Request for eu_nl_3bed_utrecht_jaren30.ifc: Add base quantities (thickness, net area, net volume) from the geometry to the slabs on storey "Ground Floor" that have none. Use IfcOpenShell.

First a look at what the model holds.

```python
import ifcopenshell
import ifcopenshell.util.element
import ifcopenshell.util.unit

model = ifcopenshell.open("eu_nl_3bed_utrecht_jaren30.ifc")
print(model.schema)
for unit_type in ("LENGTHUNIT", "AREAUNIT", "VOLUMEUNIT"):
    print(unit_type, ifcopenshell.util.unit.calculate_unit_scale(model, unit_type))
storey = next(s for s in model.by_type("IfcBuildingStorey") if s.Name == "Ground Floor")
slabs = [e for e in ifcopenshell.util.element.get_decomposition(storey) if e.is_a("IfcSlab")]
for e in sorted(slabs, key=lambda e: e.id()):
    print(e.id(), e.is_a(), e.Name, list(ifcopenshell.util.element.get_psets(e, qtos_only=True)), sep=" | ")
```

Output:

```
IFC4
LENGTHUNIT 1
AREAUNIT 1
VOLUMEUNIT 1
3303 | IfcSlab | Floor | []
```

```python
import ifcopenshell
import ifcopenshell.api.pset
import ifcopenshell.geom
import ifcopenshell.util.element
import ifcopenshell.util.shape
import ifcopenshell.util.unit

model = ifcopenshell.open("eu_nl_3bed_utrecht_jaren30.ifc")
unit_scale = ifcopenshell.util.unit.calculate_unit_scale(model)
area_scale = ifcopenshell.util.unit.calculate_unit_scale(model, "AREAUNIT")
volume_scale = ifcopenshell.util.unit.calculate_unit_scale(model, "VOLUMEUNIT")
settings = ifcopenshell.geom.settings()

storey = next(s for s in model.by_type("IfcBuildingStorey") if s.Name == "Ground Floor")
slabs = [e for e in ifcopenshell.util.element.get_decomposition(storey) if e.is_a("IfcSlab")]

for e in sorted(slabs, key=lambda e: e.id()):
    if ifcopenshell.util.element.get_psets(e, qtos_only=True, should_inherit=False):
        continue
    # Geometry comes back in metres, in the element's own axes.
    shape = ifcopenshell.geom.create_shape(settings, e)
    values = {
        "Width": ifcopenshell.util.shape.get_z(shape.geometry) / unit_scale,
        "NetArea": ifcopenshell.util.shape.get_footprint_area(shape.geometry) / area_scale,
        "NetVolume": ifcopenshell.util.shape.get_volume(shape.geometry) / volume_scale,
    }
    qto = ifcopenshell.api.pset.add_qto(model, product=e, name="Qto_SlabBaseQuantities")
    ifcopenshell.api.pset.edit_qto(model, qto=qto, properties=values)
    print(e.id(), {k: round(v, 3) for k, v in values.items()})

model.write("eu_nl_3bed_utrecht_jaren30_v2.ifc")
```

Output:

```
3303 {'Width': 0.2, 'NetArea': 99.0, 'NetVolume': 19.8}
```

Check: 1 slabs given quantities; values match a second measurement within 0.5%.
